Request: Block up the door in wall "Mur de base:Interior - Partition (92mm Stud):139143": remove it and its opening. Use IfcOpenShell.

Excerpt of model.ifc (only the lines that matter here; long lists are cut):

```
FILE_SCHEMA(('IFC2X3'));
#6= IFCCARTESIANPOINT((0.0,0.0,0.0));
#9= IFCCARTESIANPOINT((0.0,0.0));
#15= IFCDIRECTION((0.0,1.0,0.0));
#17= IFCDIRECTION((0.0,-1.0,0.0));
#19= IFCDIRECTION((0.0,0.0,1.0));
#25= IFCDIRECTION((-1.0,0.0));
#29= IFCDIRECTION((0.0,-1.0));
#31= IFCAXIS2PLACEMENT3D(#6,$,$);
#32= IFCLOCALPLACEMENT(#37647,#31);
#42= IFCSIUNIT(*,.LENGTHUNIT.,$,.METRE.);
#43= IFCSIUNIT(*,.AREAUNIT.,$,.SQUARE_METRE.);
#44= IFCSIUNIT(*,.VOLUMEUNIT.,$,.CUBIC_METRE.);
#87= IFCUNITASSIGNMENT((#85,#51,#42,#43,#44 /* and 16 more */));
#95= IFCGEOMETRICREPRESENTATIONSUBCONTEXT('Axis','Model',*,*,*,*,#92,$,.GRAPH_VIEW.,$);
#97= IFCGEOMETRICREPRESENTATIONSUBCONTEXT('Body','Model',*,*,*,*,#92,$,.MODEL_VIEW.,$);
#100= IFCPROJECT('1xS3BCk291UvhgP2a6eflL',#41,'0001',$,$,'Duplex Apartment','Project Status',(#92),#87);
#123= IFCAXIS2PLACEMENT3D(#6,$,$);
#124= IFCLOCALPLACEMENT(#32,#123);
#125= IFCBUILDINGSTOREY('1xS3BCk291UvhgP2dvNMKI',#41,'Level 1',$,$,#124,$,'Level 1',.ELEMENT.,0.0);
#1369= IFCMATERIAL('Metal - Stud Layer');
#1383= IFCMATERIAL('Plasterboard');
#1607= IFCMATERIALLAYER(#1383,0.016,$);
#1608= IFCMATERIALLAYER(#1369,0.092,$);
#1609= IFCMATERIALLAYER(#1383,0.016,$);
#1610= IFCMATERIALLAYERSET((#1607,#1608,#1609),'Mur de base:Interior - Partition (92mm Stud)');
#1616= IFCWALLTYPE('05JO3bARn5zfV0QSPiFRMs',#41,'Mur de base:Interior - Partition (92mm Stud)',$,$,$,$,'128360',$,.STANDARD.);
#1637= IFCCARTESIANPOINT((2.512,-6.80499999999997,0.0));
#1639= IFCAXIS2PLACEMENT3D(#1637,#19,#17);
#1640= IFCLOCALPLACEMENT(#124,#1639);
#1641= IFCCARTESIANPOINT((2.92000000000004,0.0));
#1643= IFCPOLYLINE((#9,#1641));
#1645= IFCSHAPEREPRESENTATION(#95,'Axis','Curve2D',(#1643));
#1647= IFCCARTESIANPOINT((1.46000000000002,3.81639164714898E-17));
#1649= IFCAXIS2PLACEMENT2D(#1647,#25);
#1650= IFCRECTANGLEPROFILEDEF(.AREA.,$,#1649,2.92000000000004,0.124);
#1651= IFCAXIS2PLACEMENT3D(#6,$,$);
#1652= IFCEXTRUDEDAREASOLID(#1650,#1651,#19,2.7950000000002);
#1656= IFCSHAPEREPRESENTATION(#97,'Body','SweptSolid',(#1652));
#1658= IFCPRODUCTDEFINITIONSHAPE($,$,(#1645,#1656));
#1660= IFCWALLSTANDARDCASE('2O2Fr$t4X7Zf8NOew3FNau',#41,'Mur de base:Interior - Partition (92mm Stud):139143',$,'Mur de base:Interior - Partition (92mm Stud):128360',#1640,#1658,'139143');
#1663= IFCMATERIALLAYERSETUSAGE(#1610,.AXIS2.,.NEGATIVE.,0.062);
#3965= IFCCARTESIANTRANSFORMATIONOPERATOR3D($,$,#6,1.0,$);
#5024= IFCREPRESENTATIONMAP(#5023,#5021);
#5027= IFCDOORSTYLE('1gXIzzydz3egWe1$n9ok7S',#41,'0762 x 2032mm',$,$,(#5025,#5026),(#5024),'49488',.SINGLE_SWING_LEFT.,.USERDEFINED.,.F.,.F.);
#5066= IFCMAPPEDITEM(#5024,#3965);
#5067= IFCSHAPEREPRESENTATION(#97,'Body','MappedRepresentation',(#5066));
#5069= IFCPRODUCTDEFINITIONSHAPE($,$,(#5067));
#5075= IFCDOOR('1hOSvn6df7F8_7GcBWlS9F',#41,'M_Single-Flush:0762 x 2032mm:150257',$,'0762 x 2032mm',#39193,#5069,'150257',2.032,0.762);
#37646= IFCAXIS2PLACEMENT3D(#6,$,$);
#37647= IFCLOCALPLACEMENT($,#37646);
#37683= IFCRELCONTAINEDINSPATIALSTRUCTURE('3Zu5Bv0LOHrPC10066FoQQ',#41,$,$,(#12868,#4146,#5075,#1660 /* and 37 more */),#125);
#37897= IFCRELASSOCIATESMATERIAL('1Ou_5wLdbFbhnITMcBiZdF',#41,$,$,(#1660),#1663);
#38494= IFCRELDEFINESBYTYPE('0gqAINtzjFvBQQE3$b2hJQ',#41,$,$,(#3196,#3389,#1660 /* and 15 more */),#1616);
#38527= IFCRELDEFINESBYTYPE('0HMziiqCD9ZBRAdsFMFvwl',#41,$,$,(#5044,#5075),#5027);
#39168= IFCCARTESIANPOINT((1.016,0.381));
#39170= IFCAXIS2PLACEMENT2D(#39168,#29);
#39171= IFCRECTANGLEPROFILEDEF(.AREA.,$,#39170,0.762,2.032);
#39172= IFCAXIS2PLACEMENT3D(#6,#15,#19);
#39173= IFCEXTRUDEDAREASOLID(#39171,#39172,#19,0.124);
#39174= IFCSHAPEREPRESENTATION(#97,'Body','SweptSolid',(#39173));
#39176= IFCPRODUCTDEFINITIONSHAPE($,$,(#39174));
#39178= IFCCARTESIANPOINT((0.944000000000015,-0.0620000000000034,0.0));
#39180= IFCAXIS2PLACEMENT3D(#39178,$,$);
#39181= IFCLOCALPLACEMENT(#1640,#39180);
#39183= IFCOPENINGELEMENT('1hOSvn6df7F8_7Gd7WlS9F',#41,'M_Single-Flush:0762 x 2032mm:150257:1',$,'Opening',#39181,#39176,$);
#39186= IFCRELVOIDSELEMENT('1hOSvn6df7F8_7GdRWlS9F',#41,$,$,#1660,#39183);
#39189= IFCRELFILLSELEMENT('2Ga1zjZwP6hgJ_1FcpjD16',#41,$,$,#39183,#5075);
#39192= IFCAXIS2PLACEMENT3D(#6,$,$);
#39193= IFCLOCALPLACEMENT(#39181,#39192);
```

```python
import ifcopenshell
import ifcopenshell.api.feature
import ifcopenshell.api.root
import ifcopenshell.geom
import ifcopenshell.util.shape

model = ifcopenshell.open("model.ifc")
settings = ifcopenshell.geom.settings()


def volume(element):
    """Net volume in cubic metres, openings subtracted."""
    shape = ifcopenshell.geom.create_shape(settings, element)
    return ifcopenshell.util.shape.get_volume(shape.geometry)


door = model.by_guid("1hOSvn6df7F8_7GcBWlS9F")
opening = door.FillsVoids[0].RelatingOpeningElement
wall = opening.VoidsElements[0].RelatingBuildingElement
before = volume(wall)

ifcopenshell.api.root.remove_product(model, product=door)
ifcopenshell.api.feature.remove_feature(model, feature=opening)

after = volume(wall)

print(f"wall volume {before:.3f} -> {after:.3f} m3")

model.write("model-out.ifc")
```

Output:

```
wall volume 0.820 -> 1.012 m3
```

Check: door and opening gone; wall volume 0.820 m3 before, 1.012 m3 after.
